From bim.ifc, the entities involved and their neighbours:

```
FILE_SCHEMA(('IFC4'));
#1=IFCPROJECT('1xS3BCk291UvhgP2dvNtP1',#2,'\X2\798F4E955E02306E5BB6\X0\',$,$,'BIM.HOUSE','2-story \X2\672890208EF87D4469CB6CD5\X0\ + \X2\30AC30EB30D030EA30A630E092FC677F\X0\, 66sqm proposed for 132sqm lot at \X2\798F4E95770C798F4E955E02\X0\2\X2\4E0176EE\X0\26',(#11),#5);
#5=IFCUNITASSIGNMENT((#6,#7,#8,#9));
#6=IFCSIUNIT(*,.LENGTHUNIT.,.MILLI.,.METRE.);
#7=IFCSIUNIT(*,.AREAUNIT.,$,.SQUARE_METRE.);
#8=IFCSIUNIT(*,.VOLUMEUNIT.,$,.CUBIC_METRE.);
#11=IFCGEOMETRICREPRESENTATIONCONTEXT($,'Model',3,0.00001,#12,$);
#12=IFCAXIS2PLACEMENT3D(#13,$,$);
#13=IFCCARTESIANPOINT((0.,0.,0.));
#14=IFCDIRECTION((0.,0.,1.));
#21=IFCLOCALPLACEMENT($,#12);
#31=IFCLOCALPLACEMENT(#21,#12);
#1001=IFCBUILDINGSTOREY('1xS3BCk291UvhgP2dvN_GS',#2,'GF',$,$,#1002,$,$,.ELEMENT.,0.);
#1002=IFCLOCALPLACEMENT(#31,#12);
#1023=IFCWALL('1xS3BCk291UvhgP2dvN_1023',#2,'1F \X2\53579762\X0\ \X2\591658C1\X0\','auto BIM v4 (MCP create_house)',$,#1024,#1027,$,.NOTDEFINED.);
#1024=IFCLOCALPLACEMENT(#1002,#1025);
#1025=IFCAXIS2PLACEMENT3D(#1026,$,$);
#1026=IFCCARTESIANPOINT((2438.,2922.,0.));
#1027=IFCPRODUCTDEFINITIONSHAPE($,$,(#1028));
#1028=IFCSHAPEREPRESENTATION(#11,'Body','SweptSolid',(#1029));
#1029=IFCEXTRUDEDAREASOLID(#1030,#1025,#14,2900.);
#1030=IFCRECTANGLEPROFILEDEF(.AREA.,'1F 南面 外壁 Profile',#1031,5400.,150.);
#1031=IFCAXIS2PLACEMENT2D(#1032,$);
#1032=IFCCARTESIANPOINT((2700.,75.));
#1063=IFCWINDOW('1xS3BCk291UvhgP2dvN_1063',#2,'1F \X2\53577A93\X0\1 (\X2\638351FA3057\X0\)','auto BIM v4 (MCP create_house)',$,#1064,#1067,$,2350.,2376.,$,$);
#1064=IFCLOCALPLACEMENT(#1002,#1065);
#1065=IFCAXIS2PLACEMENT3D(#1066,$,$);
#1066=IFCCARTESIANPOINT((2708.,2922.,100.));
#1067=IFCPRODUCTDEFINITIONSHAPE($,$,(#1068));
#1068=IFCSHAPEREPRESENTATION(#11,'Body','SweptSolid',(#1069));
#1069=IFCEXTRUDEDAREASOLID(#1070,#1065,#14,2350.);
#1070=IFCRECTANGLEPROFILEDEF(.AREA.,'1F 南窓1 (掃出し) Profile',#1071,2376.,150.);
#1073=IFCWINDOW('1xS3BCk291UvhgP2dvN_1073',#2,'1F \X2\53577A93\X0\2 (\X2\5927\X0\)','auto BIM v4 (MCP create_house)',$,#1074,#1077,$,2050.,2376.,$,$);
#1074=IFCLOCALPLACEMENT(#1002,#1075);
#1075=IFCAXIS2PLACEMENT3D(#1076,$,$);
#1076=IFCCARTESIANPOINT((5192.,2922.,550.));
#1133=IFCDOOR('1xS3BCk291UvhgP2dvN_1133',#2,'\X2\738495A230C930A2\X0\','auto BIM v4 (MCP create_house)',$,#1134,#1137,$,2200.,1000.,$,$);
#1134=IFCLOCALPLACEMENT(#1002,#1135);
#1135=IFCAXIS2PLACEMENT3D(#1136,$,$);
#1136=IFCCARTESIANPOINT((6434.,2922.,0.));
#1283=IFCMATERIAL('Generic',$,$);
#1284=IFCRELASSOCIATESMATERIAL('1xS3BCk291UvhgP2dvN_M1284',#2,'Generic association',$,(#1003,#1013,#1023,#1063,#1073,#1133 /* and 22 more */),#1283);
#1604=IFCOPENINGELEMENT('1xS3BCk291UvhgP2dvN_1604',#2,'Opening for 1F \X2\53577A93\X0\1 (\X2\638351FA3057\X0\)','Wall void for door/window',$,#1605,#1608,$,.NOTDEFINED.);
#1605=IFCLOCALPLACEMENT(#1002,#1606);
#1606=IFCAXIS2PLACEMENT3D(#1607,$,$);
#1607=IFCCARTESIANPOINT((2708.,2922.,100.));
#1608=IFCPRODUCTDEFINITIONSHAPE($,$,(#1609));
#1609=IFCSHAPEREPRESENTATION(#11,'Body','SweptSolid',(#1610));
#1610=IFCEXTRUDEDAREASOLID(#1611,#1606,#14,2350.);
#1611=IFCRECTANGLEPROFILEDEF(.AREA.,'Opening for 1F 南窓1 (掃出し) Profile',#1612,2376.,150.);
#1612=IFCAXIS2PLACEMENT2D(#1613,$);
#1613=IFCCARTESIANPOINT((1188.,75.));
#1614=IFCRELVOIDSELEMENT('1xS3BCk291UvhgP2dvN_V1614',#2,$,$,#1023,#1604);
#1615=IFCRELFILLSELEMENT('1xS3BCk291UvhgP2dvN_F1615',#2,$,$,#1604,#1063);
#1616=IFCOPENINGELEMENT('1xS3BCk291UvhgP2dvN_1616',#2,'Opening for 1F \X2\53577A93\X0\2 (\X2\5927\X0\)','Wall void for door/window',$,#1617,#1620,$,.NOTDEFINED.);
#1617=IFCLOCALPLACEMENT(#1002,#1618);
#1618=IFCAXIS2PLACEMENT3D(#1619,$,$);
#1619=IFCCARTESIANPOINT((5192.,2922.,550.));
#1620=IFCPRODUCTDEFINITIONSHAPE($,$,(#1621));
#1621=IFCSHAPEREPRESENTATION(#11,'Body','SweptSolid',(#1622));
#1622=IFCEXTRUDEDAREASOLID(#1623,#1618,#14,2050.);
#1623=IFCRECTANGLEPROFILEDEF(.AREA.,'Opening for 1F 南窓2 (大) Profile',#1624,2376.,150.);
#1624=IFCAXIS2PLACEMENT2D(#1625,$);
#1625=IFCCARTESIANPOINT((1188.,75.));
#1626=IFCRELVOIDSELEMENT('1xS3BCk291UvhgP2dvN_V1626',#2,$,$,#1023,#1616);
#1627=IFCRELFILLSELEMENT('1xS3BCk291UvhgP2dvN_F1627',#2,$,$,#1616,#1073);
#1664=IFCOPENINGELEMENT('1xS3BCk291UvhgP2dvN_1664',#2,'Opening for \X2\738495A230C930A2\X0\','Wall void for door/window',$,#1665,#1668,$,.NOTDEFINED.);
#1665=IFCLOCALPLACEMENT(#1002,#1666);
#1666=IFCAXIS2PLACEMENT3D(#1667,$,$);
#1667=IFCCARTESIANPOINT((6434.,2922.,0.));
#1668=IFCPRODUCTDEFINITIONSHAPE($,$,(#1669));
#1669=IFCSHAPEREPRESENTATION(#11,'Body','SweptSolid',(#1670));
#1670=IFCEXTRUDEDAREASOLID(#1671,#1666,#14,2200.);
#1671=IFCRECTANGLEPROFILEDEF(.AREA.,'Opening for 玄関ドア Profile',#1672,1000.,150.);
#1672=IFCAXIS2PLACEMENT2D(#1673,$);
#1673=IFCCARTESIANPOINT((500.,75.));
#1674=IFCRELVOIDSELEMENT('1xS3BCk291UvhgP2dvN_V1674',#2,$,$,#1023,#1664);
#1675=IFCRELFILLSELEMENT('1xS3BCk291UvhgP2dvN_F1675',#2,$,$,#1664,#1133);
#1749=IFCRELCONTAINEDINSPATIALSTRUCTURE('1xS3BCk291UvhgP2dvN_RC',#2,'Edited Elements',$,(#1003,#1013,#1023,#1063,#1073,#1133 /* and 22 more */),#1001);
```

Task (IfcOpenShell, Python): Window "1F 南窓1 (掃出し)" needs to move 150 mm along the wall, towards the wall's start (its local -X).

```python
import ifcopenshell
import ifcopenshell.api.geometry
import ifcopenshell.util.placement

model = ifcopenshell.open("bim.ifc")

window = model.by_guid("1xS3BCk291UvhgP2dvN_1063")
opening = window.FillsVoids[0].RelatingOpeningElement
wall = opening.VoidsElements[0].RelatingBuildingElement

wall_matrix = ifcopenshell.util.placement.get_local_placement(wall.ObjectPlacement)
shift = wall_matrix[:3, 0] * -150.0
before = ifcopenshell.util.placement.get_local_placement(window.ObjectPlacement)[:3, 3].copy()

# The window is not placed relative to its opening, so move both.
for product in (opening, window):
    matrix = ifcopenshell.util.placement.get_local_placement(product.ObjectPlacement)
    matrix[:3, 3] += shift
    ifcopenshell.api.geometry.edit_object_placement(model, product=product, matrix=matrix, is_si=False)

after = ifcopenshell.util.placement.get_local_placement(window.ObjectPlacement)[:3, 3]
print("window moved by", (after - before).round(3) + 0.0)

model.write("bim_edited.ifc")
```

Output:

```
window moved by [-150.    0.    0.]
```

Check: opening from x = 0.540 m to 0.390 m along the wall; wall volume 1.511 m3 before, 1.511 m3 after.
